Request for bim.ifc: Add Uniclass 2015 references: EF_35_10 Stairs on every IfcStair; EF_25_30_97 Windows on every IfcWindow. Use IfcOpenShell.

First a look at what the model holds.

```python
import ifcopenshell

model = ifcopenshell.open("bim.ifc")
print(model.schema)
print("classifications:", [c.Name for c in model.by_type("IfcClassification")])
for ifc_class in ("IfcDoor", "IfcRoof", "IfcStair", "IfcWall", "IfcWindow"):
    print(ifc_class, len(model.by_type(ifc_class)))
```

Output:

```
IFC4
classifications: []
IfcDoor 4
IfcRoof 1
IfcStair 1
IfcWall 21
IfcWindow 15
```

```python
import ifcopenshell
import ifcopenshell.api.classification

model = ifcopenshell.open("bim.ifc")

system = ifcopenshell.api.classification.add_classification(model, classification="Uniclass 2015")

codes = {
    "IfcStair": ("EF_35_10", "Stairs"),
    "IfcWindow": ("EF_25_30_97", "Windows"),
}
for ifc_class, (code, name) in codes.items():
    products = model.by_type(ifc_class)
    ifcopenshell.api.classification.add_reference(
        model, products=products, classification=system, identification=code, name=name
    )
    print(code, len(products))

model.write("bim_edited.ifc")
```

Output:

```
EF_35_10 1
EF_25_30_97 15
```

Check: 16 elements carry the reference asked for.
